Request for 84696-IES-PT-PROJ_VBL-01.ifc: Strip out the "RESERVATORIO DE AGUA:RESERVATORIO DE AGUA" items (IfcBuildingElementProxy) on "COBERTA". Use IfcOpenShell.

First a look at what the model holds.

```python
import ifcopenshell
import ifcopenshell.util.element

model = ifcopenshell.open("84696-IES-PT-PROJ_VBL-01.ifc")
print(model.schema)
storey = next(s for s in model.by_type("IfcBuildingStorey") if s.Name == "COBERTA")
proxies = [e for e in ifcopenshell.util.element.get_decomposition(storey) if e.is_a("IfcBuildingElementProxy")]
seen = {}
for e in proxies:
    element_type = ifcopenshell.util.element.get_type(e)
    name = element_type.Name if element_type not in (None, e) else None
    seen[name] = seen.get(name, 0) + 1
for name, count in sorted(seen.items(), key=str):
    print(count, "x", name)
```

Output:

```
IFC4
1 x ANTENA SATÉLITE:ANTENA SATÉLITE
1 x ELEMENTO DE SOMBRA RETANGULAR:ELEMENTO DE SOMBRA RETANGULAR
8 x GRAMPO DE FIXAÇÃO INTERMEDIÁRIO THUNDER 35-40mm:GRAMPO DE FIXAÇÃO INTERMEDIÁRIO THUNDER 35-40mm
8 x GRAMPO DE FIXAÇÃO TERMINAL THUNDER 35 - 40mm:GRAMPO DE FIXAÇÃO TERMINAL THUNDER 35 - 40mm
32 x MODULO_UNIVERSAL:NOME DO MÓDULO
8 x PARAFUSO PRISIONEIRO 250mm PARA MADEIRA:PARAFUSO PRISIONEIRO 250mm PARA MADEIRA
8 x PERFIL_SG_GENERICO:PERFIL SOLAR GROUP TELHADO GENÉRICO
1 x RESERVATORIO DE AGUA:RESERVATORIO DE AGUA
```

```python
import ifcopenshell
import ifcopenshell.api.root
import ifcopenshell.util.element

model = ifcopenshell.open("84696-IES-PT-PROJ_VBL-01.ifc")

storey = next(s for s in model.by_type("IfcBuildingStorey") if s.Name == "COBERTA")
proxies = [e for e in ifcopenshell.util.element.get_decomposition(storey) if e.is_a("IfcBuildingElementProxy")]
targets = [e for e in proxies if (t := ifcopenshell.util.element.get_type(e)) not in (None, e) and t.Name == "RESERVATORIO DE AGUA:RESERVATORIO DE AGUA"]

for e in targets:
    ifcopenshell.api.root.remove_product(model, product=e)
print(len(targets), "removed")

model.write("84696-IES-PT-PROJ_VBL-01_edited.ifc")
```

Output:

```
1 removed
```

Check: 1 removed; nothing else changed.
